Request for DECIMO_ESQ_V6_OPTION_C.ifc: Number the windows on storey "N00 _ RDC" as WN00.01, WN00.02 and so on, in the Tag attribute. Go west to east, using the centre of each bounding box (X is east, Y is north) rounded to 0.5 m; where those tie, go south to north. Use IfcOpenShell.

First a look at what the model holds.

```python
import ifcopenshell
import ifcopenshell.util.element
import ifcopenshell.util.placement

model = ifcopenshell.open("DECIMO_ESQ_V6_OPTION_C.ifc")
print(model.schema)
storey = next(s for s in model.by_type("IfcBuildingStorey") if s.Name == "N00 _ RDC")
windows = [e for e in ifcopenshell.util.element.get_decomposition(storey) if e.is_a("IfcWindow")]
for e in sorted(windows, key=lambda e: e.id()):
    origin = ifcopenshell.util.placement.get_local_placement(e.ObjectPlacement)[:3, 3]
    print(e.id(), e.Tag, e.Name, origin.round(2) + 0.0, sep=" | ")
```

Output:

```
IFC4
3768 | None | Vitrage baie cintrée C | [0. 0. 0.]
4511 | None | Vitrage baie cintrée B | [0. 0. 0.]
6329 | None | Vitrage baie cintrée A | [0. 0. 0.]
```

```python
import ifcopenshell
import ifcopenshell.geom
import ifcopenshell.util.element
import ifcopenshell.util.shape

model = ifcopenshell.open("DECIMO_ESQ_V6_OPTION_C.ifc")
settings = ifcopenshell.geom.settings()
settings.set("use-world-coords", True)


def centre(element):
    shape = ifcopenshell.geom.create_shape(settings, element)
    return ifcopenshell.util.shape.get_bbox_centroid(shape.geometry)


storey = next(s for s in model.by_type("IfcBuildingStorey") if s.Name == "N00 _ RDC")
windows = [e for e in ifcopenshell.util.element.get_decomposition(storey) if e.is_a("IfcWindow")]

# Insertion points can sit at a corner or the storey origin, so sort by the geometry (in metres).
centres = {e: centre(e) for e in windows}
windows.sort(key=lambda e: (round(centres[e][0] / 0.5), centres[e][1]))

for i, e in enumerate(windows, start=1):
    number = f"WN00.{i:02d}"
    e.Tag = number
    print(e.id(), number)

model.write("DECIMO_ESQ_V6_OPTION_C_edited.ifc")
```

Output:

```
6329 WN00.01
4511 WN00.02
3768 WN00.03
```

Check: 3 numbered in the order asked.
